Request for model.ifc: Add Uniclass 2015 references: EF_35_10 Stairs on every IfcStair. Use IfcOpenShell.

First a look at what the model holds.

```python
import ifcopenshell

model = ifcopenshell.open("model.ifc")
print(model.schema)
print("classifications:", [c.Name for c in model.by_type("IfcClassification")])
for ifc_class in ("IfcDoor", "IfcRoof", "IfcStair", "IfcWall", "IfcWindow"):
    print(ifc_class, len(model.by_type(ifc_class)))
```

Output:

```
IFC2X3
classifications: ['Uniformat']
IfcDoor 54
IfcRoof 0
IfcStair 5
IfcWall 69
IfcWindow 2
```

```python
import ifcopenshell
import ifcopenshell.api.classification

model = ifcopenshell.open("model.ifc")

# IFC2X3 requires Source and Edition and has no link from the project to the system.
system = model.create_entity("IfcClassification", Source="NBS", Edition="2015", Name="Uniclass 2015")

codes = {
    "IfcStair": ("EF_35_10", "Stairs"),
}
for ifc_class, (code, name) in codes.items():
    products = model.by_type(ifc_class)
    ifcopenshell.api.classification.add_reference(
        model, products=products, classification=system, identification=code, name=name
    )
    print(code, len(products))

model.write("model_updated.ifc")
```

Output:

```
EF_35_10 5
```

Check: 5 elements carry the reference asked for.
